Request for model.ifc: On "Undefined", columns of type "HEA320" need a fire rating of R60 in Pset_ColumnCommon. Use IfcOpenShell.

First a look at what the model holds.

```python
import ifcopenshell
import ifcopenshell.util.element

model = ifcopenshell.open("model.ifc")
print(model.schema)
storey = next(s for s in model.by_type("IfcBuildingStorey") if s.Name == "Undefined")
columns = [e for e in ifcopenshell.util.element.get_decomposition(storey) if e.is_a("IfcColumn")]
seen = {}
for e in columns:
    element_type = ifcopenshell.util.element.get_type(e)
    key = (element_type.Name if element_type != e and element_type else None, ifcopenshell.util.element.get_pset(e, "Pset_ColumnCommon", "FireRating"))
    seen[key] = seen.get(key, 0) + 1
for (name, value), count in sorted(seen.items(), key=str):
    print(count, "x", name, "|", value)
```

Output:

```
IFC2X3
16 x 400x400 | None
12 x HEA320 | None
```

```python
import ifcopenshell
import ifcopenshell.api.pset
import ifcopenshell.util.element

model = ifcopenshell.open("model.ifc")

storey = next(s for s in model.by_type("IfcBuildingStorey") if s.Name == "Undefined")
columns = [e for e in ifcopenshell.util.element.get_decomposition(storey) if e.is_a("IfcColumn")]

count = 0
for e in columns:
    element_type = ifcopenshell.util.element.get_type(e)
    if element_type in (None, e) or element_type.Name != "HEA320":
        continue
    found = ifcopenshell.util.element.get_pset(e, "Pset_ColumnCommon", should_inherit=False)
    if found:
        pset = model.by_id(found["id"])
        if len(ifcopenshell.util.element.get_elements_by_pset(pset)) > 1:
            pset = ifcopenshell.api.pset.unshare_pset(model, products=[e], pset=pset)[0]
    else:
        pset = ifcopenshell.api.pset.add_pset(model, product=e, name="Pset_ColumnCommon")
    ifcopenshell.api.pset.edit_pset(model, pset=pset, properties={"FireRating": "R60"})
    count += 1

print(count, "columns updated")

model.write("model_edited.ifc")
```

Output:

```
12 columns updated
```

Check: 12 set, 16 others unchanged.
